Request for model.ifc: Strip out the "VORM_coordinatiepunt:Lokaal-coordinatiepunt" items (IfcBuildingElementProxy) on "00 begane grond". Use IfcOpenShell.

First a look at what the model holds.

```python
import ifcopenshell
import ifcopenshell.util.element

model = ifcopenshell.open("model.ifc")
print(model.schema)
storey = next(s for s in model.by_type("IfcBuildingStorey") if s.Name == "00 begane grond")
proxies = [e for e in ifcopenshell.util.element.get_decomposition(storey) if e.is_a("IfcBuildingElementProxy")]
seen = {}
for e in proxies:
    element_type = ifcopenshell.util.element.get_type(e)
    name = element_type.Name if element_type not in (None, e) else None
    seen[name] = seen.get(name, 0) + 1
for name, count in sorted(seen.items(), key=str):
    print(count, "x", name)
```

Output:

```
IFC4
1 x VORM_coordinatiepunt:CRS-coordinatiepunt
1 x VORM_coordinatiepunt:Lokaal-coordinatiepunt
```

```python
import ifcopenshell
import ifcopenshell.api.root
import ifcopenshell.util.element

model = ifcopenshell.open("model.ifc")

storey = next(s for s in model.by_type("IfcBuildingStorey") if s.Name == "00 begane grond")
proxies = [e for e in ifcopenshell.util.element.get_decomposition(storey) if e.is_a("IfcBuildingElementProxy")]
targets = [e for e in proxies if (t := ifcopenshell.util.element.get_type(e)) not in (None, e) and t.Name == "VORM_coordinatiepunt:Lokaal-coordinatiepunt"]

for e in targets:
    ifcopenshell.api.root.remove_product(model, product=e)
print(len(targets), "removed")

model.write("model_rev.ifc")
```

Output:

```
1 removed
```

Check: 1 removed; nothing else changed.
